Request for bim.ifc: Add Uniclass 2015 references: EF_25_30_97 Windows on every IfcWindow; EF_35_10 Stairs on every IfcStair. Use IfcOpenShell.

First a look at what the model holds.

```python
import ifcopenshell

model = ifcopenshell.open("bim.ifc")
print(model.schema)
print("classifications:", [c.Name for c in model.by_type("IfcClassification")])
for ifc_class in ("IfcDoor", "IfcRoof", "IfcStair", "IfcWall", "IfcWindow"):
    print(ifc_class, len(model.by_type(ifc_class)))
```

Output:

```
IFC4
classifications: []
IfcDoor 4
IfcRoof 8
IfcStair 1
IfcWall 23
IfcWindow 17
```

```python
import ifcopenshell
import ifcopenshell.api.classification

model = ifcopenshell.open("bim.ifc")

system = ifcopenshell.api.classification.add_classification(model, classification="Uniclass 2015")

codes = {
    "IfcWindow": ("EF_25_30_97", "Windows"),
    "IfcStair": ("EF_35_10", "Stairs"),
}
for ifc_class, (code, name) in codes.items():
    products = model.by_type(ifc_class)
    ifcopenshell.api.classification.add_reference(
        model, products=products, classification=system, identification=code, name=name
    )
    print(code, len(products))

model.write("bim_rev.ifc")
```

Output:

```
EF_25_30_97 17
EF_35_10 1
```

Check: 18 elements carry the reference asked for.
